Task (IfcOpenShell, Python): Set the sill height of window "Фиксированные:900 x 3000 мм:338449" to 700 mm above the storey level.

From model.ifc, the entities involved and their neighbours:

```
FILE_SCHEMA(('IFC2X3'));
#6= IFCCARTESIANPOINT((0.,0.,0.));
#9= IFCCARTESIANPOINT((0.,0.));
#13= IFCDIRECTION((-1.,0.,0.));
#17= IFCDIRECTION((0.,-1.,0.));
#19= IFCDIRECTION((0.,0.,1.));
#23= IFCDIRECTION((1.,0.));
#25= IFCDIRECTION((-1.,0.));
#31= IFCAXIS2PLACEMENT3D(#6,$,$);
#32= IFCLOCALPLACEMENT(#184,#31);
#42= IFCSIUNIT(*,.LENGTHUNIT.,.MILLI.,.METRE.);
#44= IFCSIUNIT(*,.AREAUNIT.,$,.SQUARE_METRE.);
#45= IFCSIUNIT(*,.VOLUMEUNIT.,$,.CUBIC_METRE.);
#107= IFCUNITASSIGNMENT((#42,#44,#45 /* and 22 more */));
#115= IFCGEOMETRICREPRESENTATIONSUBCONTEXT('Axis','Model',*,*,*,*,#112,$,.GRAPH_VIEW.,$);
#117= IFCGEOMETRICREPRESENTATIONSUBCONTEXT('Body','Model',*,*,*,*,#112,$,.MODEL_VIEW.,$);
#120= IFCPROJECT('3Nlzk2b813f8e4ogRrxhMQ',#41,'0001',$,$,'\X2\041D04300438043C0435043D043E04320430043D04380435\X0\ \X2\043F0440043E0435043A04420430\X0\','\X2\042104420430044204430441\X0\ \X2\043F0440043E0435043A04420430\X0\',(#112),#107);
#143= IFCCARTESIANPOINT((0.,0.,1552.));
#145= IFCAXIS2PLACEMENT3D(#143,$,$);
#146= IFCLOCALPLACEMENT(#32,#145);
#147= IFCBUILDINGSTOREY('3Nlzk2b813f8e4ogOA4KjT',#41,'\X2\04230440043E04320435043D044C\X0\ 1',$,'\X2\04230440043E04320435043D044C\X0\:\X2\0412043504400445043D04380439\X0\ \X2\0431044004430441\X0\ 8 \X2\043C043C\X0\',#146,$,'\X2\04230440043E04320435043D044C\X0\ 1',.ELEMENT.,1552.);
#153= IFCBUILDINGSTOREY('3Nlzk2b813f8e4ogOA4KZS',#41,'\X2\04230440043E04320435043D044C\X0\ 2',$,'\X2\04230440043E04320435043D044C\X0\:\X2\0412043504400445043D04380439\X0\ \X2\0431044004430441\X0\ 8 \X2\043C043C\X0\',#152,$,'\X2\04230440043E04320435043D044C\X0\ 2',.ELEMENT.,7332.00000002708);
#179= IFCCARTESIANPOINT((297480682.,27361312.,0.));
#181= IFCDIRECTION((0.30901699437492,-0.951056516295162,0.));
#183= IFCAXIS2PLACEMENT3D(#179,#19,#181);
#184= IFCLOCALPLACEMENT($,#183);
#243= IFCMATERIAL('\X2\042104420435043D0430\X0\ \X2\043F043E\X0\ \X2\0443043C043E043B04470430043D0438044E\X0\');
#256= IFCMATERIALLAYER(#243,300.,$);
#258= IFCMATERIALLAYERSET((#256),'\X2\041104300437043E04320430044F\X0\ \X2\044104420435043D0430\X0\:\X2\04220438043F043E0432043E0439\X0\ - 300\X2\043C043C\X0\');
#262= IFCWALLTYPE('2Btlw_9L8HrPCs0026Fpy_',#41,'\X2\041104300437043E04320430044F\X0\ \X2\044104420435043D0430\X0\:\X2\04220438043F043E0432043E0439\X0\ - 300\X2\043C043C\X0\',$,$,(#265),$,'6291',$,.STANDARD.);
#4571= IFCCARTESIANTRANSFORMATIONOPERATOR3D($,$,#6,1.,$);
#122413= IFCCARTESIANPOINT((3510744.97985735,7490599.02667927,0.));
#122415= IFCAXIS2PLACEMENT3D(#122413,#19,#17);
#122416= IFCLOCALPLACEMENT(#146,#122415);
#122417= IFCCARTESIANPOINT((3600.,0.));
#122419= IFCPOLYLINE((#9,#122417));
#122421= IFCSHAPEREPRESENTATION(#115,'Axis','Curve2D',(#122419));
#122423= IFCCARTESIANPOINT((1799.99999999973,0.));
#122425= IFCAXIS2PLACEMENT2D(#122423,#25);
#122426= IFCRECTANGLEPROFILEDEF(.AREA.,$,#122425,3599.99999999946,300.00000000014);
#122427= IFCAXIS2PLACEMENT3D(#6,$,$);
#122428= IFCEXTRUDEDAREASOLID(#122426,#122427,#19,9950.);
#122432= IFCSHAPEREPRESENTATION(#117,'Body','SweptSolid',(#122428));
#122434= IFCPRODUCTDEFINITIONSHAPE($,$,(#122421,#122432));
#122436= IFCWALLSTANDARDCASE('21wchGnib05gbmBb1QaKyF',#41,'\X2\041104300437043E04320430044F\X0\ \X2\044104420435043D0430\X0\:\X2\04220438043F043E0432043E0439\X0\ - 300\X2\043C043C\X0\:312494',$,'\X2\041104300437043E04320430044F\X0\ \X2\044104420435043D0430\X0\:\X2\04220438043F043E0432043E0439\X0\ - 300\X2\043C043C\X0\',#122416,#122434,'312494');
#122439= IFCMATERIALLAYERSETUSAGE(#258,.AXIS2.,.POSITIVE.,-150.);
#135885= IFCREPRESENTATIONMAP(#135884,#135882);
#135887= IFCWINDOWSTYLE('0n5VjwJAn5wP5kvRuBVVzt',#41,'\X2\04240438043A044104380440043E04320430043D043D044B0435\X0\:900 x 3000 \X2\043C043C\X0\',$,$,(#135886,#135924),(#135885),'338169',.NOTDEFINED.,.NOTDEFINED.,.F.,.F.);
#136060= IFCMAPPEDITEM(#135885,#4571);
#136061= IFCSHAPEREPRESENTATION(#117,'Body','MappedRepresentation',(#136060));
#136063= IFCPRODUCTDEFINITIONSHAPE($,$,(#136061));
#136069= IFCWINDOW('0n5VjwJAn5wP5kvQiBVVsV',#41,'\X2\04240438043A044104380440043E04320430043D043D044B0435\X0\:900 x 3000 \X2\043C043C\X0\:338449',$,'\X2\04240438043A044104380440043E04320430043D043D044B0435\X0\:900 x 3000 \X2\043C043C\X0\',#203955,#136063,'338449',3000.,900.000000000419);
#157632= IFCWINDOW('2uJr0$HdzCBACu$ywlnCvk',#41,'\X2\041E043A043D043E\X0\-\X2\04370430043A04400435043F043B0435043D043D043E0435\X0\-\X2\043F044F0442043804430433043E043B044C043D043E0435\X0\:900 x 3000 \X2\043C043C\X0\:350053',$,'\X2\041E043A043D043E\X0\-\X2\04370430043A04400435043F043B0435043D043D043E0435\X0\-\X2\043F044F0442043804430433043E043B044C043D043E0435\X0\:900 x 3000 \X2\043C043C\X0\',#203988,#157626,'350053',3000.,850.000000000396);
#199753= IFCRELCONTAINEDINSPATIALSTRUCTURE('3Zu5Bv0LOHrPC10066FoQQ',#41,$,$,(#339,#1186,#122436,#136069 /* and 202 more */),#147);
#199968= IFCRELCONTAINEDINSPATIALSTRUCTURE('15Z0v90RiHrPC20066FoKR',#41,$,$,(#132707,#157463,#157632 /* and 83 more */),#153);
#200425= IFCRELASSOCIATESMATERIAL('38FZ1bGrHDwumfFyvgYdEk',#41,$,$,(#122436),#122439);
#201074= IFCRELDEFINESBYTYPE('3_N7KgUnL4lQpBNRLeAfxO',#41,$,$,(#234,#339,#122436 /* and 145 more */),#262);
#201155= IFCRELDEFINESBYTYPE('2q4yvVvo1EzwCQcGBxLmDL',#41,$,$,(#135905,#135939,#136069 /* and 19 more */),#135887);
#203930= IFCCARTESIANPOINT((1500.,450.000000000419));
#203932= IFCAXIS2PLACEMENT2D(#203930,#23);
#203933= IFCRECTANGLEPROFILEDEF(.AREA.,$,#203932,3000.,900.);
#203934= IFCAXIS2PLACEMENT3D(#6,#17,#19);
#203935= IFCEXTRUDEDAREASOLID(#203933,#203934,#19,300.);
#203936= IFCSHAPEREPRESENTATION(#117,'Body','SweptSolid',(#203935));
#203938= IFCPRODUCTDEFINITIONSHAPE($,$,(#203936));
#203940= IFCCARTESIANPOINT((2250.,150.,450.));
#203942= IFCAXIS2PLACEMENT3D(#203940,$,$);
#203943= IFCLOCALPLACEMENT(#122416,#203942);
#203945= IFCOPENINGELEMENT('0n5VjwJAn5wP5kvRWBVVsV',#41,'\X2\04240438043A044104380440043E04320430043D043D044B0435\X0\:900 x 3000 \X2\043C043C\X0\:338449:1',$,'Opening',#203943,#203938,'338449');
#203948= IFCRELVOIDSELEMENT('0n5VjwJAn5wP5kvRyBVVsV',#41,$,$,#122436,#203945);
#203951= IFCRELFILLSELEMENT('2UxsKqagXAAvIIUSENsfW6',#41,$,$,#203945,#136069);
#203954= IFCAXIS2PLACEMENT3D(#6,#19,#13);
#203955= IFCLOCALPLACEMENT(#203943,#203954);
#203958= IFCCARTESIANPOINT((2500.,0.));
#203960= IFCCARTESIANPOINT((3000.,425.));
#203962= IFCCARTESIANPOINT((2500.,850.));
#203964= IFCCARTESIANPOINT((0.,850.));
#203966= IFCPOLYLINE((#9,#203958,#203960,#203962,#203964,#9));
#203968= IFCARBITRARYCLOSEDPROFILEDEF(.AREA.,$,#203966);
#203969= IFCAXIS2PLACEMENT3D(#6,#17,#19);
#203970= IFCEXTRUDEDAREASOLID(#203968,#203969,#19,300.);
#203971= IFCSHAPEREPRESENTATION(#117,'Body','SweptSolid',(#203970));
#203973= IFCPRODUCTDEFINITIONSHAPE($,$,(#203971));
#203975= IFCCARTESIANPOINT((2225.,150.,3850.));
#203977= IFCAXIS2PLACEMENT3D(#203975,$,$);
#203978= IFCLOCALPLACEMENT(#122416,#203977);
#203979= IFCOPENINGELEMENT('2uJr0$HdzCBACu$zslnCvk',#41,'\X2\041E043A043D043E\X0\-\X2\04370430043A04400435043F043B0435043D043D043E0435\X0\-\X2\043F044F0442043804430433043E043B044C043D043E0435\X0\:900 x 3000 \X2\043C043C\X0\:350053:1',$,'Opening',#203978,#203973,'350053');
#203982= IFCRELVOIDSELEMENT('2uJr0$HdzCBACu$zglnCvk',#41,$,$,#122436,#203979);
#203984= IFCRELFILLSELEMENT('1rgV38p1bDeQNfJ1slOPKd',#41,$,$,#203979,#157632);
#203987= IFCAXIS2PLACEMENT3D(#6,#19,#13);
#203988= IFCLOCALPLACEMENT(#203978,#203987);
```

```python
import numpy as np
import ifcopenshell
import ifcopenshell.api.geometry
import ifcopenshell.geom
import ifcopenshell.util.element
import ifcopenshell.util.placement
import ifcopenshell.util.shape
import ifcopenshell.util.unit

model = ifcopenshell.open("model.ifc")
unit_scale = ifcopenshell.util.unit.calculate_unit_scale(model)

window = model.by_guid("0n5VjwJAn5wP5kvQiBVVsV")
opening = window.FillsVoids[0].RelatingOpeningElement
storey = ifcopenshell.util.element.get_container(window, ifc_class="IfcBuildingStorey")
level = ifcopenshell.util.placement.get_local_placement(storey.ObjectPlacement)[2, 3]

# The opening's origin need not be at the sill, so measure its lowest point.
shape = ifcopenshell.geom.create_shape(ifcopenshell.geom.settings(), opening)
bottom = ifcopenshell.util.shape.get_shape_bottom_elevation(shape, shape.geometry) / unit_scale
dz = level + 700.0 - bottom

shift = np.array([0.0, 0.0, dz])
# The window is placed relative to its opening, so it follows when the opening moves.
matrix = ifcopenshell.util.placement.get_local_placement(opening.ObjectPlacement)
matrix[:3, 3] += shift
ifcopenshell.api.geometry.edit_object_placement(
    model, product=opening, matrix=matrix, is_si=False, should_transform_children=True
)

print(f"moved by {dz * unit_scale:+.3f} m")

model.write("model_edited.ifc")
```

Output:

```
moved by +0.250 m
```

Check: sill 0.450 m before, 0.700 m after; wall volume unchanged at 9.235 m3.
